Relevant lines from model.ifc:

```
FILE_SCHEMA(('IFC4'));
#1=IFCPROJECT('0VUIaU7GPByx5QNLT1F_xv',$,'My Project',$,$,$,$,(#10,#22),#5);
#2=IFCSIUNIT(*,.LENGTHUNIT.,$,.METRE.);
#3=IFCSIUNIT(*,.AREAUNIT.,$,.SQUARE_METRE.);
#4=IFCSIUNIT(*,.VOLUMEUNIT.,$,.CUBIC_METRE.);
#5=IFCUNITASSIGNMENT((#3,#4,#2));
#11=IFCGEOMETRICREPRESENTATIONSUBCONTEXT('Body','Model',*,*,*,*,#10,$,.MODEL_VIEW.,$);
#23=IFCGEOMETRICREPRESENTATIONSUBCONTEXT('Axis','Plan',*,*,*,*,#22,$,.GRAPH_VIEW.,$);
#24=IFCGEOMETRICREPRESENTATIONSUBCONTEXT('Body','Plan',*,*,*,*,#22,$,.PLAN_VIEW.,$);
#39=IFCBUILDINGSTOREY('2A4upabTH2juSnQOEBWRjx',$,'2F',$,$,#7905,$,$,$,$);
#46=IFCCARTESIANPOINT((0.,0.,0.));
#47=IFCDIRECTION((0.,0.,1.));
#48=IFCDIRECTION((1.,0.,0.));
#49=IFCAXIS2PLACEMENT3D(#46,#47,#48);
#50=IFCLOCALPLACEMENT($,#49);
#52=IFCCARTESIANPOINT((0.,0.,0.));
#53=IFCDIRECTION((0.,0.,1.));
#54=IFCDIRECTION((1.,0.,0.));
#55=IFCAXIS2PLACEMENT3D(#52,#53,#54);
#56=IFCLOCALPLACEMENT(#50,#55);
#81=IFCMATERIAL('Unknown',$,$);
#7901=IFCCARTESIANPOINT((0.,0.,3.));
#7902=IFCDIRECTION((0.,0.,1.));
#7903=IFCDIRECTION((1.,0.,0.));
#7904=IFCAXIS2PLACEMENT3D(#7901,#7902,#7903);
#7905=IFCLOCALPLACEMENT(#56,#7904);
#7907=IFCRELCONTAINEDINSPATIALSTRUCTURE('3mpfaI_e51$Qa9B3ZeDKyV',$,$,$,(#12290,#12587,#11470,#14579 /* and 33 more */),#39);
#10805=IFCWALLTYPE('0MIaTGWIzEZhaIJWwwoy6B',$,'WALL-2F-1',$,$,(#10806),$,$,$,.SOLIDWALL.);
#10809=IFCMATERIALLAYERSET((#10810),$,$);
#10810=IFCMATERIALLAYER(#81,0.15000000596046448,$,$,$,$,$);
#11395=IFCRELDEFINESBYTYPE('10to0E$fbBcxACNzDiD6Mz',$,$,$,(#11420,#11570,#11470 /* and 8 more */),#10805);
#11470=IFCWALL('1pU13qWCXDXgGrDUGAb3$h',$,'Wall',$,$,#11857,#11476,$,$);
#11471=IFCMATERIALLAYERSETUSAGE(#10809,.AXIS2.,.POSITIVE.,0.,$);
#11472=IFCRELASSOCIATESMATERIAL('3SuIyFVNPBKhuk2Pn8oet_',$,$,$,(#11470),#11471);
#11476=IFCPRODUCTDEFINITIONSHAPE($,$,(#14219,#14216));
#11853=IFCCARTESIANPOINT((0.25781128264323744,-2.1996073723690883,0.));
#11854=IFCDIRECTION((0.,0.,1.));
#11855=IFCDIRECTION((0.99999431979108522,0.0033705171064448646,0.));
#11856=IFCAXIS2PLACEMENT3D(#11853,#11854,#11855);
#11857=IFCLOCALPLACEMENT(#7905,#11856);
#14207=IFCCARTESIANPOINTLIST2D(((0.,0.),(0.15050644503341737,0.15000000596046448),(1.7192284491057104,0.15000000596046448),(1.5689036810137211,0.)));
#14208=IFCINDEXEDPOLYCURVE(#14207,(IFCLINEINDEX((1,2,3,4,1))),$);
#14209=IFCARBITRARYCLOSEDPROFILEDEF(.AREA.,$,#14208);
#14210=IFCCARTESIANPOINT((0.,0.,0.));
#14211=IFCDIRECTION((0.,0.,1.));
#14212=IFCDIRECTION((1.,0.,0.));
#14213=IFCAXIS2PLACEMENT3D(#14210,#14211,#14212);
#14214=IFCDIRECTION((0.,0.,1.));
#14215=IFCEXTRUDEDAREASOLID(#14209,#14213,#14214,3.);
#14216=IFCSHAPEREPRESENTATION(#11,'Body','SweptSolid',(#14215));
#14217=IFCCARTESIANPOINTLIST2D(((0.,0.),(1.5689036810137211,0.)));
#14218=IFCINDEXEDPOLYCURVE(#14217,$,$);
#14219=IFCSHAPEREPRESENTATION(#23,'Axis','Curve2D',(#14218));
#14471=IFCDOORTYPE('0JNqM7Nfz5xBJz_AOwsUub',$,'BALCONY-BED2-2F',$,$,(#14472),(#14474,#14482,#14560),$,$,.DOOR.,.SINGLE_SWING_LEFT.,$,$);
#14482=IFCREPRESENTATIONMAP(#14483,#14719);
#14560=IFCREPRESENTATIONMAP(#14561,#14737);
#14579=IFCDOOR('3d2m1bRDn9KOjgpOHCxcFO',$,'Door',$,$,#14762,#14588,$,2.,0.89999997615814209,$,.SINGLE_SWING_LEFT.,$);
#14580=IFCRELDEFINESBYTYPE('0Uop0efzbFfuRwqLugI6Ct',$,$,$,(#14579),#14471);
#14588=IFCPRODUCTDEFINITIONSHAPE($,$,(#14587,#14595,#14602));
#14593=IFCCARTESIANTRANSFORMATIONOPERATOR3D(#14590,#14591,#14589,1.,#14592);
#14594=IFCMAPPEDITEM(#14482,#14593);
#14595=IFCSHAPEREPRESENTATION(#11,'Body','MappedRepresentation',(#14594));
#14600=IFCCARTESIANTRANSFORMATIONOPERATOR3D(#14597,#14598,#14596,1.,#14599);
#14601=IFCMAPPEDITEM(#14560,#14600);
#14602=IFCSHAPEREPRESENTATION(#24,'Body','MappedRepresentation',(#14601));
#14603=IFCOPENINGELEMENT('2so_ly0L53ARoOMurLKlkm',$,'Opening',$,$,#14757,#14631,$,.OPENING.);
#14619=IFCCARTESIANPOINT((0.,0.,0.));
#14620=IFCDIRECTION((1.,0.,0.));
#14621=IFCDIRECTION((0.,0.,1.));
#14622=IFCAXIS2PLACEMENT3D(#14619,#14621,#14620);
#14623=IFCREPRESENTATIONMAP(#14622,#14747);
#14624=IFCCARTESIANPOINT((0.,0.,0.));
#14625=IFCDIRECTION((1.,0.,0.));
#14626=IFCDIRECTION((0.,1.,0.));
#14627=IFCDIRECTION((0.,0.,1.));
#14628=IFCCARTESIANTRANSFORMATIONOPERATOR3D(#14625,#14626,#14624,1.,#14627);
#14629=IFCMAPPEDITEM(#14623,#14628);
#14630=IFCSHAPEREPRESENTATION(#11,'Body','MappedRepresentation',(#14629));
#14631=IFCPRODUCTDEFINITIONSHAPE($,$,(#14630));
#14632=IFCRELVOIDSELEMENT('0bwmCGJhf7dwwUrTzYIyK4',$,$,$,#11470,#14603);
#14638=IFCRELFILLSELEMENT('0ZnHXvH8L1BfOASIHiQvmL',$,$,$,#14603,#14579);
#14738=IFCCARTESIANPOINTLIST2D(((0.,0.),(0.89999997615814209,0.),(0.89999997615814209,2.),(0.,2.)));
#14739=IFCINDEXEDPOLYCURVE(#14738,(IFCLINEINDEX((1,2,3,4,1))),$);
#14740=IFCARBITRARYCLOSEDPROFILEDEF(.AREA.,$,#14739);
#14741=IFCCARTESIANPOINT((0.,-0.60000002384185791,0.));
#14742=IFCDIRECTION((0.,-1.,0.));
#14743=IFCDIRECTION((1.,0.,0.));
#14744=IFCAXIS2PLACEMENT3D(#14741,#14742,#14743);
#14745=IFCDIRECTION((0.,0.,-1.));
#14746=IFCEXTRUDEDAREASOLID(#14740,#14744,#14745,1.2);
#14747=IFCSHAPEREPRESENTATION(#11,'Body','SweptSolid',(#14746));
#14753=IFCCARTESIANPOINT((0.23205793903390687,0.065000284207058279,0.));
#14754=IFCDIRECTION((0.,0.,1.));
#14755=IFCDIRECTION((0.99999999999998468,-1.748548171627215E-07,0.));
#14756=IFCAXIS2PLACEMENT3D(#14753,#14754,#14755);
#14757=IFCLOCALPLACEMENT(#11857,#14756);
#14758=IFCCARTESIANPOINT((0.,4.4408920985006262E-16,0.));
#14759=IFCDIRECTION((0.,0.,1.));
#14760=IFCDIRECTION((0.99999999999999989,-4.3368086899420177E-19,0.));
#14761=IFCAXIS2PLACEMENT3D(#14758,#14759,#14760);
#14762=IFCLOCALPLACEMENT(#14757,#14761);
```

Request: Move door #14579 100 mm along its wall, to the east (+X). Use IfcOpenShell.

```python
import ifcopenshell
import ifcopenshell.api.geometry
import ifcopenshell.util.placement
import ifcopenshell.util.unit

model = ifcopenshell.open("model.ifc")
unit_scale = ifcopenshell.util.unit.calculate_unit_scale(model)

door = model.by_guid("3d2m1bRDn9KOjgpOHCxcFO")
opening = door.FillsVoids[0].RelatingOpeningElement
wall = opening.VoidsElements[0].RelatingBuildingElement

wall_matrix = ifcopenshell.util.placement.get_local_placement(wall.ObjectPlacement)
shift = wall_matrix[:3, 0] * 0.1 / unit_scale
before = ifcopenshell.util.placement.get_local_placement(door.ObjectPlacement)[:3, 3].copy()

# The door is placed relative to its opening, so it follows when the opening moves.
matrix = ifcopenshell.util.placement.get_local_placement(opening.ObjectPlacement)
matrix[:3, 3] += shift
ifcopenshell.api.geometry.edit_object_placement(
    model, product=opening, matrix=matrix, is_si=False, should_transform_children=True
)

after = ifcopenshell.util.placement.get_local_placement(door.ObjectPlacement)[:3, 3]
print("door moved by", (after - before).round(3) + 0.0)

model.write("model-out.ifc")
```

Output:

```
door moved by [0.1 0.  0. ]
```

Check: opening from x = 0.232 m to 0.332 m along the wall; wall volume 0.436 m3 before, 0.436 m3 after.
